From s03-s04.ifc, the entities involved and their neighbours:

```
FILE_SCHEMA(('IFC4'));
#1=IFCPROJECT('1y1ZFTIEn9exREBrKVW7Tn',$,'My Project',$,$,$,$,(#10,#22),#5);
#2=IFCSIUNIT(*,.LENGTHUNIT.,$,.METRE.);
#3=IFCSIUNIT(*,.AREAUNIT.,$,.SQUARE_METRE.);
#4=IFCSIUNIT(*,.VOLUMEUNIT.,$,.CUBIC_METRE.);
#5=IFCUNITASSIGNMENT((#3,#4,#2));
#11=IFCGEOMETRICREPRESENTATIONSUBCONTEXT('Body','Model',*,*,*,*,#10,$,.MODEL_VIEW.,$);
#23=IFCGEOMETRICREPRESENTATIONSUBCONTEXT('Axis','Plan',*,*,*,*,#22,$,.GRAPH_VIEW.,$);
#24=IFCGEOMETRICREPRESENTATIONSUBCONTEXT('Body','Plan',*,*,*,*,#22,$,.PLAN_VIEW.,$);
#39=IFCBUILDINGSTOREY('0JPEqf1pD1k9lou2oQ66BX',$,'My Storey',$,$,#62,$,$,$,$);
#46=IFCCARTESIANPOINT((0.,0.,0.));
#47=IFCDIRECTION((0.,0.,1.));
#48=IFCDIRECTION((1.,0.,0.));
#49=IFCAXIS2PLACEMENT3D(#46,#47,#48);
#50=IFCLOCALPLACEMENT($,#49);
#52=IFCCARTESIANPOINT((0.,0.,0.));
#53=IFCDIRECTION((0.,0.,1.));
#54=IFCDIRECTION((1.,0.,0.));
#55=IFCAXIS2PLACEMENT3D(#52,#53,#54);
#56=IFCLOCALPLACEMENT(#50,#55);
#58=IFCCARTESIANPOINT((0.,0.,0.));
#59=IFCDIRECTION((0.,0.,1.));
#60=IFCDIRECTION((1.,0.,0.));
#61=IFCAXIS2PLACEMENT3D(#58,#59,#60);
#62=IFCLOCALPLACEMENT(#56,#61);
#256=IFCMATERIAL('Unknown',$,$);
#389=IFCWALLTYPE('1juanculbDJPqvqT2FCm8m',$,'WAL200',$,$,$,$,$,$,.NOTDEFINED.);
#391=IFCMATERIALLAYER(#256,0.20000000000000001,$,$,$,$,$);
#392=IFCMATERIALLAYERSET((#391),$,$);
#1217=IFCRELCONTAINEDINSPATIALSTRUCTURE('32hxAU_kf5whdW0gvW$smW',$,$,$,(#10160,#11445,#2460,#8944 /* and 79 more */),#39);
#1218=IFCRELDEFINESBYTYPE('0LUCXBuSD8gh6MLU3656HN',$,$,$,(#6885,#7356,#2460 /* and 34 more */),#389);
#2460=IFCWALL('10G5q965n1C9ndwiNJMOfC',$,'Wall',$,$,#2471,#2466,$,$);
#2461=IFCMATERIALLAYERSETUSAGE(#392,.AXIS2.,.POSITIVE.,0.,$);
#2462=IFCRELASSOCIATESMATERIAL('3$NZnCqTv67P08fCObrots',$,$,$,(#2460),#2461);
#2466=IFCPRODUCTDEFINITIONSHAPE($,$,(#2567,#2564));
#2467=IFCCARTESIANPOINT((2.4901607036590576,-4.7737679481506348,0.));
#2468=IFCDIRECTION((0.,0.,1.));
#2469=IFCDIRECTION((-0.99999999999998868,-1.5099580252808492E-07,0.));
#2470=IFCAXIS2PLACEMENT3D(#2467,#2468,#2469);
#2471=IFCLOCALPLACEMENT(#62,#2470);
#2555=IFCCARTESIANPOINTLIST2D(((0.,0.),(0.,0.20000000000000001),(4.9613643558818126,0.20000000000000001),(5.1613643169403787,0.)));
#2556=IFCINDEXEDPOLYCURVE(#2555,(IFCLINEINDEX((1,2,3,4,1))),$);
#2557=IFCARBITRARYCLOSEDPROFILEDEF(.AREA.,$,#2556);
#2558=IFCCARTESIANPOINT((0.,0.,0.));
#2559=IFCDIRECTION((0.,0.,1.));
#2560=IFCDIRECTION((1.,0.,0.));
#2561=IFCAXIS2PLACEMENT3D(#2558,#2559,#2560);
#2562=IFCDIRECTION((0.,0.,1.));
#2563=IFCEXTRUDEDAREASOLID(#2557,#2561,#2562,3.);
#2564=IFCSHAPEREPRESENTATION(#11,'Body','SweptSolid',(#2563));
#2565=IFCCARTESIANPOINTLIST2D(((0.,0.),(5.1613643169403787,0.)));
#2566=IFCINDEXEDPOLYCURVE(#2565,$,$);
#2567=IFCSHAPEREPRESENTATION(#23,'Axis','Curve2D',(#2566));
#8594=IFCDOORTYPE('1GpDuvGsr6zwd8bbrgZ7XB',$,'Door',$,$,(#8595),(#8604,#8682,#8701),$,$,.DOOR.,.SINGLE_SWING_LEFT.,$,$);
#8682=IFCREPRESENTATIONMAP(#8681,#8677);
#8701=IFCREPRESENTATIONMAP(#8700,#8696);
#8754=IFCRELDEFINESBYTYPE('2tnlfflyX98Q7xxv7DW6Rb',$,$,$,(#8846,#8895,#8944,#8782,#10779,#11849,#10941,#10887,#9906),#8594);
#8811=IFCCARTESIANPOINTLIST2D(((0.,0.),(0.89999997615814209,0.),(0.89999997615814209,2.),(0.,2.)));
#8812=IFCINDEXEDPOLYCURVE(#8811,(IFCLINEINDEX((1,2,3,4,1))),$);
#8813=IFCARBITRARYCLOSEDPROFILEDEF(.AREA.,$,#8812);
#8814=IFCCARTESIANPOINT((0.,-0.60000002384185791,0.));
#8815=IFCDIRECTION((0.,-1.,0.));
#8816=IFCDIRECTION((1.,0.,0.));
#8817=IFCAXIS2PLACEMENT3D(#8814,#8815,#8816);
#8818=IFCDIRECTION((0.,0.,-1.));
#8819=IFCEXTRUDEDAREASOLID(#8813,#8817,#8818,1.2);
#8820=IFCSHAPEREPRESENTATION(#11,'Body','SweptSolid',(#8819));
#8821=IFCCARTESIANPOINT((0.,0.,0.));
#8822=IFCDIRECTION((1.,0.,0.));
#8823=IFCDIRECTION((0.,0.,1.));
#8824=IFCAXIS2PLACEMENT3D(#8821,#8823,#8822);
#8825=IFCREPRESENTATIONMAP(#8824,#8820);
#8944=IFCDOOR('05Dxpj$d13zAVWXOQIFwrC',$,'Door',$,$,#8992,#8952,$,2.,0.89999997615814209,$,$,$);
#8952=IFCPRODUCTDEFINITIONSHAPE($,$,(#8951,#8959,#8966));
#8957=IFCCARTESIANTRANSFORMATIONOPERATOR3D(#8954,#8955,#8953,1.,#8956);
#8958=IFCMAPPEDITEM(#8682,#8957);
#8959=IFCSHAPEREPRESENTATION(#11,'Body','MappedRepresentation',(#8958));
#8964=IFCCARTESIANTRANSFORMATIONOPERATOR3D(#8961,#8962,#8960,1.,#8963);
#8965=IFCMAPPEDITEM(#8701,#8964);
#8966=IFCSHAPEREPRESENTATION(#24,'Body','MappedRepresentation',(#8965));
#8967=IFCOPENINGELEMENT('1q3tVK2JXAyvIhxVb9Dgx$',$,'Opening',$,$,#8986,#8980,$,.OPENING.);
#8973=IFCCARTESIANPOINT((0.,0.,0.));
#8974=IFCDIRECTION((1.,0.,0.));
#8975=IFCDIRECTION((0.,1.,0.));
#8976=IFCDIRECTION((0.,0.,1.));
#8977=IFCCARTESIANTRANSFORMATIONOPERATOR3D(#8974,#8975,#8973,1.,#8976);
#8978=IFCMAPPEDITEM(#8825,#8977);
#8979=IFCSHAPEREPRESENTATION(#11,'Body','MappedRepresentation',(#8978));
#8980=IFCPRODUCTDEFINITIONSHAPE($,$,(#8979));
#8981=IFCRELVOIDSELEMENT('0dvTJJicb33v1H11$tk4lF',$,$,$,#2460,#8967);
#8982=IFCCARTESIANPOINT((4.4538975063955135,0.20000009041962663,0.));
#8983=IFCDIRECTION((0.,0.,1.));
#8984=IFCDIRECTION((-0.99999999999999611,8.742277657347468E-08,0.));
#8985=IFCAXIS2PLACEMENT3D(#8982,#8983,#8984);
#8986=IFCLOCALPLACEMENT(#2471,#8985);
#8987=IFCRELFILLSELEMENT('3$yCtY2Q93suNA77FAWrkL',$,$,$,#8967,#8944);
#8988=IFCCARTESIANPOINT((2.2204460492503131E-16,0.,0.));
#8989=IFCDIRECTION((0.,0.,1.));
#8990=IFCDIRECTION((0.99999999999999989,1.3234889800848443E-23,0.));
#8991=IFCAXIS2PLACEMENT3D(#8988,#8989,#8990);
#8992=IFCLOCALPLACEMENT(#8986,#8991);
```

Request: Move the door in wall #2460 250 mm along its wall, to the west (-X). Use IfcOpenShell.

```python
import ifcopenshell
import ifcopenshell.api.geometry
import ifcopenshell.util.placement
import ifcopenshell.util.unit

model = ifcopenshell.open("s03-s04.ifc")
unit_scale = ifcopenshell.util.unit.calculate_unit_scale(model)

door = model.by_guid("05Dxpj$d13zAVWXOQIFwrC")
opening = door.FillsVoids[0].RelatingOpeningElement
wall = opening.VoidsElements[0].RelatingBuildingElement

wall_matrix = ifcopenshell.util.placement.get_local_placement(wall.ObjectPlacement)
shift = wall_matrix[:3, 0] * 0.25 / unit_scale
before = ifcopenshell.util.placement.get_local_placement(door.ObjectPlacement)[:3, 3].copy()

# The door is placed relative to its opening, so it follows when the opening moves.
matrix = ifcopenshell.util.placement.get_local_placement(opening.ObjectPlacement)
matrix[:3, 3] += shift
ifcopenshell.api.geometry.edit_object_placement(
    model, product=opening, matrix=matrix, is_si=False, should_transform_children=True
)

after = ifcopenshell.util.placement.get_local_placement(door.ObjectPlacement)[:3, 3]
print("door moved by", (after - before).round(3) + 0.0)

model.write("s03-s04-out.ifc")
```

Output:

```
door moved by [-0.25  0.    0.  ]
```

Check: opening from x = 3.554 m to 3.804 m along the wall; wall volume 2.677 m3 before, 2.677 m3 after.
